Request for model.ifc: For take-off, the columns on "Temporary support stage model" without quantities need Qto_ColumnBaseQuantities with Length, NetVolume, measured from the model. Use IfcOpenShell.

First a look at what the model holds.

```python
import ifcopenshell
import ifcopenshell.util.element
import ifcopenshell.util.unit

model = ifcopenshell.open("model.ifc")
print(model.schema)
for unit_type in ("LENGTHUNIT", "AREAUNIT", "VOLUMEUNIT"):
    print(unit_type, ifcopenshell.util.unit.calculate_unit_scale(model, unit_type))
storey = next(s for s in model.by_type("IfcBuildingStorey") if s.Name == "Temporary support stage model")
columns = [e for e in ifcopenshell.util.element.get_decomposition(storey) if e.is_a("IfcColumn")]
for e in sorted(columns, key=lambda e: e.id()):
    print(e.id(), e.is_a(), e.Name, list(ifcopenshell.util.element.get_psets(e, qtos_only=True)), sep=" | ")
```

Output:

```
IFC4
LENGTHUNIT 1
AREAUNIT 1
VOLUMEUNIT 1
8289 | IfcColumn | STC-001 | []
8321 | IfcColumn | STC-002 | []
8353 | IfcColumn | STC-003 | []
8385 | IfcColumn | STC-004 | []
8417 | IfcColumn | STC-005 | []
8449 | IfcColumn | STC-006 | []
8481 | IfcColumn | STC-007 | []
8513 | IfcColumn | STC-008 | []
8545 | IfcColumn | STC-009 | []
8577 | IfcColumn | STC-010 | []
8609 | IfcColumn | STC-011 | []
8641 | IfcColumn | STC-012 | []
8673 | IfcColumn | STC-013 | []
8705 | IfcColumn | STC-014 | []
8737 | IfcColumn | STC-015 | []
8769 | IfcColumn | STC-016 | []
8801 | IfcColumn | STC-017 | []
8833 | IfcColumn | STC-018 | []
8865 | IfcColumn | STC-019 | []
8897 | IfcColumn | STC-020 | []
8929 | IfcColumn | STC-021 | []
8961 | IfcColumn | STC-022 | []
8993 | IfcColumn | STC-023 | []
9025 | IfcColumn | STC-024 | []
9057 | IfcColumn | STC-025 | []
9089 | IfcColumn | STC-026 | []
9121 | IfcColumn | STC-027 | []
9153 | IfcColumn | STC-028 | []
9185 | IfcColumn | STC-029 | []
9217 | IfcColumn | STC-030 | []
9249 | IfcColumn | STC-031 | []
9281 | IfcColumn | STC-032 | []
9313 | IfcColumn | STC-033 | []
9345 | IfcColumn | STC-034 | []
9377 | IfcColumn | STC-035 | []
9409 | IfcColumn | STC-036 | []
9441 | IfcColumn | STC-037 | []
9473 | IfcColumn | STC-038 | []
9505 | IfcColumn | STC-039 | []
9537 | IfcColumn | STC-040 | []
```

```python
import ifcopenshell
import ifcopenshell.api.pset
import ifcopenshell.geom
import ifcopenshell.util.element
import ifcopenshell.util.shape
import ifcopenshell.util.unit

model = ifcopenshell.open("model.ifc")
unit_scale = ifcopenshell.util.unit.calculate_unit_scale(model)
volume_scale = ifcopenshell.util.unit.calculate_unit_scale(model, "VOLUMEUNIT")
settings = ifcopenshell.geom.settings()

storey = next(s for s in model.by_type("IfcBuildingStorey") if s.Name == "Temporary support stage model")
columns = [e for e in ifcopenshell.util.element.get_decomposition(storey) if e.is_a("IfcColumn")]

for e in sorted(columns, key=lambda e: e.id()):
    if ifcopenshell.util.element.get_psets(e, qtos_only=True, should_inherit=False):
        continue
    # Geometry comes back in metres, in the element's own axes.
    shape = ifcopenshell.geom.create_shape(settings, e)
    values = {
        "Length": ifcopenshell.util.shape.get_z(shape.geometry) / unit_scale,
        "NetVolume": ifcopenshell.util.shape.get_volume(shape.geometry) / volume_scale,
    }
    qto = ifcopenshell.api.pset.add_qto(model, product=e, name="Qto_ColumnBaseQuantities")
    ifcopenshell.api.pset.edit_qto(model, qto=qto, properties=values)
    print(e.id(), {k: round(v, 3) for k, v in values.items()})

model.write("model_rev.ifc")
```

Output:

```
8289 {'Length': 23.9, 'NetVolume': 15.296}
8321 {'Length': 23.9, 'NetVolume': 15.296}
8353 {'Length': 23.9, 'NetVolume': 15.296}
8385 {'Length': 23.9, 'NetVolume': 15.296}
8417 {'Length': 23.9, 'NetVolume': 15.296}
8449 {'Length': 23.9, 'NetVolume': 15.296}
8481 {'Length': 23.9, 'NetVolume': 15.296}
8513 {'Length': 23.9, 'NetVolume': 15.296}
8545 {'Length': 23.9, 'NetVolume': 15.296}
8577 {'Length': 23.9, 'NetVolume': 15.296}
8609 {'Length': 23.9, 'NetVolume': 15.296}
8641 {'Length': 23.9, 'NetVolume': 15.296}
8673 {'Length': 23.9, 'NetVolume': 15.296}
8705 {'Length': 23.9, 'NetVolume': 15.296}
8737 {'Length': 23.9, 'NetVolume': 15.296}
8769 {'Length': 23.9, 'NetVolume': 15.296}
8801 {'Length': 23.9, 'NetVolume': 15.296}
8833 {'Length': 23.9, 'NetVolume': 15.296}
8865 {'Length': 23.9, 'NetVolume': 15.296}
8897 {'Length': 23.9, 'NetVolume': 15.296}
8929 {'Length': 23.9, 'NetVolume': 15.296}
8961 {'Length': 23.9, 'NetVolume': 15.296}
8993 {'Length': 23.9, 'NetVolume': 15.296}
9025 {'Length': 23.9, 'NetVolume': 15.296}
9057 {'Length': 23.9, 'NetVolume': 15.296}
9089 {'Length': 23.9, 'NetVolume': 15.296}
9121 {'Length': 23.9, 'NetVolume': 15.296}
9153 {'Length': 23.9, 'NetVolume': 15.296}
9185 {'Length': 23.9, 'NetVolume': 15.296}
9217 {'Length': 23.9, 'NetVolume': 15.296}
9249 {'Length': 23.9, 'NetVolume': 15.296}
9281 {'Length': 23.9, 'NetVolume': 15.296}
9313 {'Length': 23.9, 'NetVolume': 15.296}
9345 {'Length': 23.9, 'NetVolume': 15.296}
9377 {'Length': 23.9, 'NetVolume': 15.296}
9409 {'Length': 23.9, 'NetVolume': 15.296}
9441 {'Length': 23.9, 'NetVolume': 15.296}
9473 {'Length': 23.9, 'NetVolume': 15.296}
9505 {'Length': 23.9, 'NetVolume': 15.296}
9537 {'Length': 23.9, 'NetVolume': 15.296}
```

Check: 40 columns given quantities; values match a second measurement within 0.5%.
